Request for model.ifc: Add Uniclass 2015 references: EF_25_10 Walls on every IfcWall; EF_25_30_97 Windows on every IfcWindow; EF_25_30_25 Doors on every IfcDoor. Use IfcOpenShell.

First a look at what the model holds.

```python
import ifcopenshell

model = ifcopenshell.open("model.ifc")
print(model.schema)
print("classifications:", [c.Name for c in model.by_type("IfcClassification")])
for ifc_class in ("IfcDoor", "IfcRoof", "IfcStair", "IfcWall", "IfcWindow"):
    print(ifc_class, len(model.by_type(ifc_class)))
```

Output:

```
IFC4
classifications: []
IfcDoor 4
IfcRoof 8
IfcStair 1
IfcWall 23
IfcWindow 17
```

```python
import ifcopenshell
import ifcopenshell.api.classification

model = ifcopenshell.open("model.ifc")

system = ifcopenshell.api.classification.add_classification(model, classification="Uniclass 2015")

codes = {
    "IfcWall": ("EF_25_10", "Walls"),
    "IfcWindow": ("EF_25_30_97", "Windows"),
    "IfcDoor": ("EF_25_30_25", "Doors"),
}
for ifc_class, (code, name) in codes.items():
    products = model.by_type(ifc_class)
    ifcopenshell.api.classification.add_reference(
        model, products=products, classification=system, identification=code, name=name
    )
    print(code, len(products))

model.write("model_updated.ifc")
```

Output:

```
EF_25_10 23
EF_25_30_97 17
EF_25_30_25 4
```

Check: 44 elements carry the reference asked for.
